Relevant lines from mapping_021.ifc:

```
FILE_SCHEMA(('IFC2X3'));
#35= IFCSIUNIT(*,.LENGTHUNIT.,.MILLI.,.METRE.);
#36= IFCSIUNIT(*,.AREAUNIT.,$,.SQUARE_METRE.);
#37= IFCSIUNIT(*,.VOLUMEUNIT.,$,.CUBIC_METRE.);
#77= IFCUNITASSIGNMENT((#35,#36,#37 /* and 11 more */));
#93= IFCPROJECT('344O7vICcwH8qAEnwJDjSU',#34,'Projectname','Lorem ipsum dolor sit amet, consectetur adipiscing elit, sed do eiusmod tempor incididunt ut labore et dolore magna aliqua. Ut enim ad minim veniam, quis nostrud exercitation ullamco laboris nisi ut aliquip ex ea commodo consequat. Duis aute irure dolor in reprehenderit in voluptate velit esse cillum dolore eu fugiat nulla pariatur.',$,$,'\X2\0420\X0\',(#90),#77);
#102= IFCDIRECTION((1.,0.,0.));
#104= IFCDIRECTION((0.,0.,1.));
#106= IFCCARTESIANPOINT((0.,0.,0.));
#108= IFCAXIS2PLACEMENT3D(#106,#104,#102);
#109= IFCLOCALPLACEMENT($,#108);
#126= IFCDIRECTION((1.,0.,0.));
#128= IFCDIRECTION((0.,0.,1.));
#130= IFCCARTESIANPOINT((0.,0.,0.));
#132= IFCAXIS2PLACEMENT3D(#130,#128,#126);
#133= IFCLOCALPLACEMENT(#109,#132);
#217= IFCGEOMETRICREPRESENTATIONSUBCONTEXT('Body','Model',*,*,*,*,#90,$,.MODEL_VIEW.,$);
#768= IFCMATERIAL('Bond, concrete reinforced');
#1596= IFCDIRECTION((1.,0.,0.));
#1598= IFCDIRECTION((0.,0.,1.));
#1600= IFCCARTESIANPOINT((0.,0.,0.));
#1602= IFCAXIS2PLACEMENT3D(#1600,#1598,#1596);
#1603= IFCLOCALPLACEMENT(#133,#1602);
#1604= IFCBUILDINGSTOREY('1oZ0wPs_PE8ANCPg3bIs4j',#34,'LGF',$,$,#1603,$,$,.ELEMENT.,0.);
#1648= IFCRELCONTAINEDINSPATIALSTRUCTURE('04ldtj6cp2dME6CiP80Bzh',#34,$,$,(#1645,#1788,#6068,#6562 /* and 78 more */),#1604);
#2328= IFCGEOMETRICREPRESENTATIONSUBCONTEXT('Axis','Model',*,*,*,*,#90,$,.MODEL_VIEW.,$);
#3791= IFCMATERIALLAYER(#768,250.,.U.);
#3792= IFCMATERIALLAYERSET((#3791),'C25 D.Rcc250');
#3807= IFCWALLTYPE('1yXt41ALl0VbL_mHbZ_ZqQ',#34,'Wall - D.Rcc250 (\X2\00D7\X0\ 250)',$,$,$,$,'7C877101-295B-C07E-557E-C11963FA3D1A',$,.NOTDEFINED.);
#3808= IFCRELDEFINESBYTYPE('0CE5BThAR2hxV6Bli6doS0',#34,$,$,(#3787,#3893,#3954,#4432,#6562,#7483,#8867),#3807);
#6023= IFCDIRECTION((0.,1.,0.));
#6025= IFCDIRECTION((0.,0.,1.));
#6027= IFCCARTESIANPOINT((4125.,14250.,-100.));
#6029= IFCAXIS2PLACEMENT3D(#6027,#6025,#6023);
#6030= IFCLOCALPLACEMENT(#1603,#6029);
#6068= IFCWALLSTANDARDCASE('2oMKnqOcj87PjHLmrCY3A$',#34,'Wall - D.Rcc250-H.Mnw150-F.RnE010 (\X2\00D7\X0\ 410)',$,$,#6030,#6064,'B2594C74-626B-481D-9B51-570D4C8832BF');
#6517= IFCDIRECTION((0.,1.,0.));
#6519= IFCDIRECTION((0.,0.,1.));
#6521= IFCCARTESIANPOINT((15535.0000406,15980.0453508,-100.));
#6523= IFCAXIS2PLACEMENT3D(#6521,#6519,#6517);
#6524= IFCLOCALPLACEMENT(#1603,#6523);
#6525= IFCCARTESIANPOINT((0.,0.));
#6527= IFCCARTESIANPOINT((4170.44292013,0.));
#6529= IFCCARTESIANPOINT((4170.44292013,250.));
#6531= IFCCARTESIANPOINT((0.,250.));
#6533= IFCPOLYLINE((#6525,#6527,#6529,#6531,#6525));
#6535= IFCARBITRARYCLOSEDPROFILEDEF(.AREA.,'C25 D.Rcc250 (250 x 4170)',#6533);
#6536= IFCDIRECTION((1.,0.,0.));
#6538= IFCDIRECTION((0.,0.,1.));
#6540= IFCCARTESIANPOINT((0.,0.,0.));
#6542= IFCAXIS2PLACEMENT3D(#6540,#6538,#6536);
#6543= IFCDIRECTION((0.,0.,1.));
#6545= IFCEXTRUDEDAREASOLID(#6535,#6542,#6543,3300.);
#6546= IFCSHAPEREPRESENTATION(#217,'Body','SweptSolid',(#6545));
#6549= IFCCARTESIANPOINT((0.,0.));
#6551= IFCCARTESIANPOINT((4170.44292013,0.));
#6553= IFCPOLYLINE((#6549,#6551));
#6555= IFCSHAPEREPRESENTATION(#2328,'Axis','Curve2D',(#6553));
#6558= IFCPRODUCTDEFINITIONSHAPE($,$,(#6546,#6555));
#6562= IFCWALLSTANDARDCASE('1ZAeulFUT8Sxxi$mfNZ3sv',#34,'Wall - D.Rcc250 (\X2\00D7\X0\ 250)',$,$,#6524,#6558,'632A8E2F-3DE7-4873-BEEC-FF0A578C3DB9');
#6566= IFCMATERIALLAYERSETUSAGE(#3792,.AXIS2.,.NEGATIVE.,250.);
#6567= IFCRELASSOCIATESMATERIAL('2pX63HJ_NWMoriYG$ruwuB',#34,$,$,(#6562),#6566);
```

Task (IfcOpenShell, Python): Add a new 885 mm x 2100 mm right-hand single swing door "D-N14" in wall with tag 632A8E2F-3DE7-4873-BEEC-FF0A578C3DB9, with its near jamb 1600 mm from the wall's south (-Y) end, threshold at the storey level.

```python
import numpy as np
import ifcopenshell
import ifcopenshell.api.feature
import ifcopenshell.api.geometry
import ifcopenshell.api.root
import ifcopenshell.api.spatial
import ifcopenshell.api.type
import ifcopenshell.geom
import ifcopenshell.util.element
import ifcopenshell.util.placement
import ifcopenshell.util.representation
import ifcopenshell.util.shape
import ifcopenshell.util.unit

model = ifcopenshell.open("mapping_021.ifc")
unit_scale = ifcopenshell.util.unit.calculate_unit_scale(model)
settings = ifcopenshell.geom.settings()


def volume(element):
    """Net volume in cubic metres, openings subtracted."""
    shape = ifcopenshell.geom.create_shape(settings, element)
    return ifcopenshell.util.shape.get_volume(shape.geometry)


wall = model.by_guid("1ZAeulFUT8Sxxi$mfNZ3sv")
storey = ifcopenshell.util.element.get_container(wall, ifc_class="IfcBuildingStorey")
context = ifcopenshell.util.representation.get_context(model, "Model", "Body", "MODEL_VIEW")
before = volume(wall)

width, height, from_end, sill = 0.885, 2.1, 1.6, 0.0  # metres

# The wall runs along its own X axis, and the end named is its -X end.
wall_shape = ifcopenshell.geom.create_shape(settings, wall)
x, y, z = ifcopenshell.util.shape.get_vertices(wall_shape.geometry).T
start = x.min() + from_end
face, thickness = float(y.min()), float(y.max() - y.min())
wall_matrix = ifcopenshell.util.placement.get_local_placement(wall.ObjectPlacement)
level = ifcopenshell.util.placement.get_local_placement(storey.ObjectPlacement)[2, 3]


def in_wall(x, y):
    """Placement at x, y metres in the wall's axes, at sill height."""
    matrix = wall_matrix.copy()
    matrix[:, 3] = wall_matrix @ np.array([x / unit_scale, y / unit_scale, 0.0, 1.0])
    matrix[2, 3] = level + sill / unit_scale
    return matrix


# Opening: a box that overshoots both wall faces by 50 mm.
opening = ifcopenshell.api.root.create_entity(model, ifc_class="IfcOpeningElement")
box = ifcopenshell.api.geometry.add_wall_representation(
    model, context=context, length=width, height=height, thickness=thickness + 0.1
)
ifcopenshell.api.geometry.assign_representation(model, product=opening, representation=box)
ifcopenshell.api.geometry.edit_object_placement(model, product=opening, matrix=in_wall(start, face - 0.05), is_si=False)
ifcopenshell.api.feature.add_feature(model, feature=opening, element=wall)

door = ifcopenshell.api.root.create_entity(model, ifc_class="IfcDoor", name="D-N14")
door.OverallWidth, door.OverallHeight = width / unit_scale, height / unit_scale
body = ifcopenshell.api.geometry.add_door_representation(
    model,
    context=context,
    overall_width=door.OverallWidth,
    overall_height=door.OverallHeight,
    operation_type="SINGLE_SWING_RIGHT",
    lining_properties={"LiningDepth": thickness / unit_scale, "ThresholdDepth": thickness / unit_scale},
)
ifcopenshell.api.geometry.assign_representation(model, product=door, representation=body)
ifcopenshell.api.spatial.assign_container(model, products=[door], relating_structure=storey)
fills = ifcopenshell.api.feature.add_filling(model, opening=opening, element=door)
fills.OwnerHistory = door.OwnerHistory  # required in IFC2X3

# IFC2X3 keeps the operation on the door style.
style = ifcopenshell.api.root.create_entity(model, ifc_class="IfcDoorStyle", name="D-N14")
style.OperationType, style.ConstructionType = "SINGLE_SWING_RIGHT", "NOTDEFINED"
style.ParameterTakesPrecedence = style.Sizeable = False
ifcopenshell.api.type.assign_type(model, related_objects=[door], relating_type=style)

# The lining spans the wall, so the door starts at the wall face.
ifcopenshell.api.geometry.edit_object_placement(model, product=door, matrix=in_wall(start, face), is_si=False)

after = volume(wall)

print(f"wall volume {before:.3f} -> {after:.3f} m3")

model.write("mapping_021_rev.ifc")
```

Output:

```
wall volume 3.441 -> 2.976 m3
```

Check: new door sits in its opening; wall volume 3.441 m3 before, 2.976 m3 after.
